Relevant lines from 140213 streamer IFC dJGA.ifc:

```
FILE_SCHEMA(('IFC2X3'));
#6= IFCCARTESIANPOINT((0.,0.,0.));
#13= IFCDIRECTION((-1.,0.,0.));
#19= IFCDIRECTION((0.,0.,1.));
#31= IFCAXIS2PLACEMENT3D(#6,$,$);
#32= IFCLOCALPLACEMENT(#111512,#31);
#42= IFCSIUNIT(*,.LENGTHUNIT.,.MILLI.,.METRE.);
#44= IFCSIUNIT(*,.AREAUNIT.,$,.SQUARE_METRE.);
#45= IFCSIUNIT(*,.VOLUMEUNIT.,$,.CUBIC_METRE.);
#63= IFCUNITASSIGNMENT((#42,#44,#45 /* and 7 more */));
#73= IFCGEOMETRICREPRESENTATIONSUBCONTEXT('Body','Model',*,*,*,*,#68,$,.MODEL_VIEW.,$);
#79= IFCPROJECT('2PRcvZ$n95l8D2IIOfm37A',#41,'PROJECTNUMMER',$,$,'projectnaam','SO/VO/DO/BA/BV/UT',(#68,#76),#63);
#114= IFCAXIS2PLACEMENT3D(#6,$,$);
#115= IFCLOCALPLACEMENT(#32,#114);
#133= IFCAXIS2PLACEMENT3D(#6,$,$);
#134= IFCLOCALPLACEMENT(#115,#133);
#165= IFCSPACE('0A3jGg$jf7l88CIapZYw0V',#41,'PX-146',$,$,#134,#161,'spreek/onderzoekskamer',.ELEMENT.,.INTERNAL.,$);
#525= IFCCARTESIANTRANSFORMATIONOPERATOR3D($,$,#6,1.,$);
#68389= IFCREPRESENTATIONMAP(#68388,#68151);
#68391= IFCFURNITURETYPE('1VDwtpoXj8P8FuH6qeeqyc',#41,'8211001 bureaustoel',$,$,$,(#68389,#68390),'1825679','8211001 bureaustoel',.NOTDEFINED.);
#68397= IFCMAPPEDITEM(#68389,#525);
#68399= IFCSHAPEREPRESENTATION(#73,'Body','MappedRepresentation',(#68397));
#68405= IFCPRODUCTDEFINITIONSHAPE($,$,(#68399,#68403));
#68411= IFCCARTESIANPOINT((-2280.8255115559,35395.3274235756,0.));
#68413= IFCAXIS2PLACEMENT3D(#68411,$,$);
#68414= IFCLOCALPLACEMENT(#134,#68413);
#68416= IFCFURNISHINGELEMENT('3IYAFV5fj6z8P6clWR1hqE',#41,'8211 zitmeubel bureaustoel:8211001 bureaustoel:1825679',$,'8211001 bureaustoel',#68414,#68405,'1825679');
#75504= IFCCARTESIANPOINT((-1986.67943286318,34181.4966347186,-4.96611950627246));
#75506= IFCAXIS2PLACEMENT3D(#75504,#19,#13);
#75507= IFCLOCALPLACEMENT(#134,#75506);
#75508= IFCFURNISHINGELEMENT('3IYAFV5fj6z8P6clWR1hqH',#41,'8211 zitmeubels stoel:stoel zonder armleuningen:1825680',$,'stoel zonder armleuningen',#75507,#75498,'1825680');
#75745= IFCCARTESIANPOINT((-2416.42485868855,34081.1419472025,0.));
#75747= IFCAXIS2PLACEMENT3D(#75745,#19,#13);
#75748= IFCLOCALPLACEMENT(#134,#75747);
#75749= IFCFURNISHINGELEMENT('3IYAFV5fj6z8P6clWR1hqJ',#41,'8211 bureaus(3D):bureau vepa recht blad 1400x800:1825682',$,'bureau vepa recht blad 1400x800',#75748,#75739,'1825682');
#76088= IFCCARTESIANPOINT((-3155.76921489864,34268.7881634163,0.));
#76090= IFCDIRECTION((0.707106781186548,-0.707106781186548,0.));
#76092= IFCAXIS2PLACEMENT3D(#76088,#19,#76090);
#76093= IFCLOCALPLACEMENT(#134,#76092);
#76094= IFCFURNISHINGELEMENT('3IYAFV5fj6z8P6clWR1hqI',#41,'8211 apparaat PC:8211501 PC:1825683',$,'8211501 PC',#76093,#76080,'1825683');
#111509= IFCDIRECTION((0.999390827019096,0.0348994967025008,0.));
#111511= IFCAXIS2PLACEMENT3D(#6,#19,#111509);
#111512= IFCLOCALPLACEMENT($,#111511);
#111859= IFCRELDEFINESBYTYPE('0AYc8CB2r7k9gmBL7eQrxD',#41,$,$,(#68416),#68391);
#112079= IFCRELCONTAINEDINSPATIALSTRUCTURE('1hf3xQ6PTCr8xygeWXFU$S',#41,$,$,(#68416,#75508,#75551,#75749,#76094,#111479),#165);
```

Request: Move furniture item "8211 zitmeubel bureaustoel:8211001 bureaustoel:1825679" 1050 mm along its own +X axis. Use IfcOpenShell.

```python
import ifcopenshell
import ifcopenshell.api.geometry
import ifcopenshell.util.placement

model = ifcopenshell.open("140213 streamer IFC dJGA.ifc")

item = model.by_guid("3IYAFV5fj6z8P6clWR1hqE")
matrix = ifcopenshell.util.placement.get_local_placement(item.ObjectPlacement)
matrix[:3, 3] += matrix[:3, 0] * 1050.0
ifcopenshell.api.geometry.edit_object_placement(model, product=item, matrix=matrix, is_si=False)

print(ifcopenshell.util.placement.get_local_placement(item.ObjectPlacement).round(3) + 0.0)

model.write("140213 streamer IFC dJGA_rev.ifc")
```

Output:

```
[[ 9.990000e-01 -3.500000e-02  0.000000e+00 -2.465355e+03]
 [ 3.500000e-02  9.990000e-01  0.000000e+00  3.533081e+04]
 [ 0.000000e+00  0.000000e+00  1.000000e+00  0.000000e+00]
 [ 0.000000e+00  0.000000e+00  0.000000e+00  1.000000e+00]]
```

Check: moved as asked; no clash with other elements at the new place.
